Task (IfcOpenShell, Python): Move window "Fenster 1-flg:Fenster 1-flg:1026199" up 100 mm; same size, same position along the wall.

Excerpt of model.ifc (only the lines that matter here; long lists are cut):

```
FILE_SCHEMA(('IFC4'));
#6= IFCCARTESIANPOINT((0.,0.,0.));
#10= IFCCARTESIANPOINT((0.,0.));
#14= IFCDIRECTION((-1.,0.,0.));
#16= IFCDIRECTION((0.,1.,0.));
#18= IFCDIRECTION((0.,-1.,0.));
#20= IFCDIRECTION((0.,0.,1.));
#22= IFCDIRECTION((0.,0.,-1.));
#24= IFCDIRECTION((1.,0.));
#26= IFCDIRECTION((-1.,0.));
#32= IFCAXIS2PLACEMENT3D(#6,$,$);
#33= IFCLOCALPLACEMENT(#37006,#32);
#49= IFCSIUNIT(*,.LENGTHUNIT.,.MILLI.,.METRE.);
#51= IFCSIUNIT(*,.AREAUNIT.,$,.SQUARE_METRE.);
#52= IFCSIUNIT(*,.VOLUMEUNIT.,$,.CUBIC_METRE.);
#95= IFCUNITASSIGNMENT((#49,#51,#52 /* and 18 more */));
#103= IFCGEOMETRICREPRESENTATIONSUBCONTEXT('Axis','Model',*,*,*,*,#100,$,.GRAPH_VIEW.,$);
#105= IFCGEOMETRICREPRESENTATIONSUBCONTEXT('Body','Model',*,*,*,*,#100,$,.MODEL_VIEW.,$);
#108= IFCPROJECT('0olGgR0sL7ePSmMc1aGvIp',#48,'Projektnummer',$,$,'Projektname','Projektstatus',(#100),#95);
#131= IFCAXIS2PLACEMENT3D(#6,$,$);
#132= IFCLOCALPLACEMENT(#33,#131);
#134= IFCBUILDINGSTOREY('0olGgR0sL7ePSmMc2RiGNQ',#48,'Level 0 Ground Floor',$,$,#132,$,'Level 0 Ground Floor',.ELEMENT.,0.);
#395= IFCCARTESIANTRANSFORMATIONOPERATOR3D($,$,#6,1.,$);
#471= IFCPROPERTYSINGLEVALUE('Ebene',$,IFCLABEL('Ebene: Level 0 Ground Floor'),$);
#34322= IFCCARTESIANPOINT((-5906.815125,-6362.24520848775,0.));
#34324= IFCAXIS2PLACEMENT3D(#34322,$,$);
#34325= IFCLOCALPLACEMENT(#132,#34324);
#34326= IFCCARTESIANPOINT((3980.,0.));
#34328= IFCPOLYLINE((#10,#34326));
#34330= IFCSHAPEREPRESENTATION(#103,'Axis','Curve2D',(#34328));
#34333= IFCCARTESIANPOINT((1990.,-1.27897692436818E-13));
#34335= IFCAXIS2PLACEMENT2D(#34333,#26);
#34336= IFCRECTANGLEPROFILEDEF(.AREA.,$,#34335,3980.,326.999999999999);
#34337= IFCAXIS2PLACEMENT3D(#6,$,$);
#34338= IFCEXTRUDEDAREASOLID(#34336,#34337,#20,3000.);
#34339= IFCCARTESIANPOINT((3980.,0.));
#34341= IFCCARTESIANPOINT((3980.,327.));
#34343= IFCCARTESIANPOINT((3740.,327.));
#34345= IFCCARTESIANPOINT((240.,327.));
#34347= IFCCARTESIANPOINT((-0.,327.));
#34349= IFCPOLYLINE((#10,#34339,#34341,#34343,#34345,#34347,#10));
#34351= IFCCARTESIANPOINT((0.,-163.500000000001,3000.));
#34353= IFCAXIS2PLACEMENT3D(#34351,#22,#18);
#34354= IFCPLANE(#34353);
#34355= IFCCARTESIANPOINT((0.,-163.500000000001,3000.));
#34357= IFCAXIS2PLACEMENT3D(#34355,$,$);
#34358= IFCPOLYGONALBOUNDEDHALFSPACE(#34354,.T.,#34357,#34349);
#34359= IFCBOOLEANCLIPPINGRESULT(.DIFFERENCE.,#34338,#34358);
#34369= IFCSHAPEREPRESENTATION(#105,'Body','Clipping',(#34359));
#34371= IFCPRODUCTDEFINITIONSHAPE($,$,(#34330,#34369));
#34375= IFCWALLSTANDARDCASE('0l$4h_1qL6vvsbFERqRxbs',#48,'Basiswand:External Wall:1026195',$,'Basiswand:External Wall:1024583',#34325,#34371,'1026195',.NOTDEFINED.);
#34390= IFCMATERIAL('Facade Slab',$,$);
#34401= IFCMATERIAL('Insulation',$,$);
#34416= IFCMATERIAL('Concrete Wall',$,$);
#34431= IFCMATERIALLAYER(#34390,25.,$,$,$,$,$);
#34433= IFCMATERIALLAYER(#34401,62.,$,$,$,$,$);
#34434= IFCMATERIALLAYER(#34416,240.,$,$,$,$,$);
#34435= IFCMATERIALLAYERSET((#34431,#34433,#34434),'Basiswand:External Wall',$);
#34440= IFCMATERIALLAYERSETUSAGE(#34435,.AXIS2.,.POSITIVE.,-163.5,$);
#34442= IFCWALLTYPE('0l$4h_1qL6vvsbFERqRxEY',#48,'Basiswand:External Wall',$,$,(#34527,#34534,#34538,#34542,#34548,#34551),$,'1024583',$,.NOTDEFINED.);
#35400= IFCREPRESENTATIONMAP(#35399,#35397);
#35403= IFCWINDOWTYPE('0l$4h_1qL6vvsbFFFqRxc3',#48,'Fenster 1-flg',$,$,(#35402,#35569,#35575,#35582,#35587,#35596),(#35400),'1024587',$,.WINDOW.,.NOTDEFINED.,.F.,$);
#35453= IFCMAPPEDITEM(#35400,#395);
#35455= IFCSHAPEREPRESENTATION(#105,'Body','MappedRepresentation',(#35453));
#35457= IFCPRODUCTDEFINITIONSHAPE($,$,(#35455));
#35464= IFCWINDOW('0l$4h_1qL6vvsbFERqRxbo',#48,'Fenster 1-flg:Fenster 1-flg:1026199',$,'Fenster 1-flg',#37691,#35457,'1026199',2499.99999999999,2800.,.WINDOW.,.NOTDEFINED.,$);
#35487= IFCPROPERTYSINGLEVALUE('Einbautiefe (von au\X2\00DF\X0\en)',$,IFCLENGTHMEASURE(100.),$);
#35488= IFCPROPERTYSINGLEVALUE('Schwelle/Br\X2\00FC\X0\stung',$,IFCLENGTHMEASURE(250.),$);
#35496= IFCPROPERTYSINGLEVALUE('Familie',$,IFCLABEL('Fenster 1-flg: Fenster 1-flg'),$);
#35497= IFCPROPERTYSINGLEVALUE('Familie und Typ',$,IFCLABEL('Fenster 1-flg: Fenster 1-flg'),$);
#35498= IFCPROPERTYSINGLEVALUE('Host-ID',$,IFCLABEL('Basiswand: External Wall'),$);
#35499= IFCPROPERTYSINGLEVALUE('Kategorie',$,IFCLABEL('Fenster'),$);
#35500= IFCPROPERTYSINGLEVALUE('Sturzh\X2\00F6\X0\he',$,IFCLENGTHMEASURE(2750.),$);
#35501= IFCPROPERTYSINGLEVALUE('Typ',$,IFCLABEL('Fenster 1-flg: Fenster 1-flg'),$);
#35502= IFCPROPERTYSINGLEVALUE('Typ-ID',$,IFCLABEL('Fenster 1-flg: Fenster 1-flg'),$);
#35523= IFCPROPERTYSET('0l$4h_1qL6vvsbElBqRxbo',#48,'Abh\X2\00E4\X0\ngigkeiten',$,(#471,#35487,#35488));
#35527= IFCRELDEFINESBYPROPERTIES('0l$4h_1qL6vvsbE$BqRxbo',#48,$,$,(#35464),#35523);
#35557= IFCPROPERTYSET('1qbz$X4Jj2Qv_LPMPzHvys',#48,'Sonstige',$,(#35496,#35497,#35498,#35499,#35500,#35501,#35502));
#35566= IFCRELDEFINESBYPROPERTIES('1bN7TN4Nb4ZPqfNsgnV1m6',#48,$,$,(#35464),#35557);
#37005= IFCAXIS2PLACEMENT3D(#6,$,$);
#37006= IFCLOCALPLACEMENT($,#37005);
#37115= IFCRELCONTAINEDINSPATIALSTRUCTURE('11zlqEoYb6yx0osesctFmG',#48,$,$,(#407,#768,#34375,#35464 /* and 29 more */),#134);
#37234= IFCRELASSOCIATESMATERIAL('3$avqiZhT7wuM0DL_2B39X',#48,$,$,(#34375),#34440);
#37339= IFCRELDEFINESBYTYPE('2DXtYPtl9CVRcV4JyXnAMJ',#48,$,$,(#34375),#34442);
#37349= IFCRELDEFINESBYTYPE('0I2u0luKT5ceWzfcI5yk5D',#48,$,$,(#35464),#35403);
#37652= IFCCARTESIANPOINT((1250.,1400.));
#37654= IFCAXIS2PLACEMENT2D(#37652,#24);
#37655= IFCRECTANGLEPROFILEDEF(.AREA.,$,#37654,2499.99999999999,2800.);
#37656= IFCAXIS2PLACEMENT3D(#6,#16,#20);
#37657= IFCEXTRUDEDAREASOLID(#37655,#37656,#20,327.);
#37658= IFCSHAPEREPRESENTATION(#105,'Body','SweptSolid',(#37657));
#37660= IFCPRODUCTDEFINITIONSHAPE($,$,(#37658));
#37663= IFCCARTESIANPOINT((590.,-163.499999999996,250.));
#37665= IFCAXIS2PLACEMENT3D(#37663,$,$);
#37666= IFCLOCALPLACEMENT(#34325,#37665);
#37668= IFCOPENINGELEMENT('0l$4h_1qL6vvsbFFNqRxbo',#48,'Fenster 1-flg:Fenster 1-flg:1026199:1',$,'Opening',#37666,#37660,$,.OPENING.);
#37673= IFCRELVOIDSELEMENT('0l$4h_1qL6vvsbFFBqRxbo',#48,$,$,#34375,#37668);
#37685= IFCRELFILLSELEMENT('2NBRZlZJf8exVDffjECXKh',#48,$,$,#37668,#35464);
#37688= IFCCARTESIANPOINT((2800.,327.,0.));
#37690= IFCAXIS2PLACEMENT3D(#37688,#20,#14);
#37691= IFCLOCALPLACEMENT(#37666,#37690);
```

```python
import numpy as np
import ifcopenshell
import ifcopenshell.api.geometry
import ifcopenshell.api.pset
import ifcopenshell.util.element
import ifcopenshell.util.placement
import ifcopenshell.util.unit

model = ifcopenshell.open("model.ifc")
unit_scale = ifcopenshell.util.unit.calculate_unit_scale(model)

window = model.by_guid("0l$4h_1qL6vvsbFERqRxbo")
opening = window.FillsVoids[0].RelatingOpeningElement
dz = 0.1 / unit_scale

shift = np.array([0.0, 0.0, dz])
# The window is placed relative to its opening, so it follows when the opening moves.
matrix = ifcopenshell.util.placement.get_local_placement(opening.ObjectPlacement)
matrix[:3, 3] += shift
ifcopenshell.api.geometry.edit_object_placement(
    model, product=opening, matrix=matrix, is_si=False, should_transform_children=True
)

# Keep the stored heights in step.
pset = model.by_id(ifcopenshell.util.element.get_pset(window, "Abhängigkeiten", should_inherit=False)["id"])
ifcopenshell.api.pset.edit_pset(model, pset=pset, properties={
    "Schwelle/Brüstung": model.create_entity("IfcLengthMeasure", ifcopenshell.util.element.get_pset(window, "Abhängigkeiten", "Schwelle/Brüstung") + dz),
})
pset = model.by_id(ifcopenshell.util.element.get_pset(window, "Sonstige", should_inherit=False)["id"])
ifcopenshell.api.pset.edit_pset(model, pset=pset, properties={
    "Sturzhöhe": model.create_entity("IfcLengthMeasure", ifcopenshell.util.element.get_pset(window, "Sonstige", "Sturzhöhe") + dz),
})

print(f"moved by {dz * unit_scale:+.3f} m")

model.write("model_edited.ifc")
```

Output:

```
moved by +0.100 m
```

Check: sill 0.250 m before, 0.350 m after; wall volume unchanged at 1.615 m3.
